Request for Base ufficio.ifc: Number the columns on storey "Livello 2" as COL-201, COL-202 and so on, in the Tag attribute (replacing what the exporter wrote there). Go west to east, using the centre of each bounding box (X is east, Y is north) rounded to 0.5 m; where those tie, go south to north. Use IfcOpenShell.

First a look at what the model holds.

```python
import ifcopenshell
import ifcopenshell.util.element
import ifcopenshell.util.placement

model = ifcopenshell.open("Base ufficio.ifc")
print(model.schema)
storey = next(s for s in model.by_type("IfcBuildingStorey") if s.Name == "Livello 2")
columns = [e for e in ifcopenshell.util.element.get_decomposition(storey) if e.is_a("IfcColumn")]
for e in sorted(columns, key=lambda e: e.id()):
    origin = ifcopenshell.util.placement.get_local_placement(e.ObjectPlacement)[:3, 3]
    print(e.id(), e.Tag, e.Name, origin.round(2) + 0.0, sep=" | ")
```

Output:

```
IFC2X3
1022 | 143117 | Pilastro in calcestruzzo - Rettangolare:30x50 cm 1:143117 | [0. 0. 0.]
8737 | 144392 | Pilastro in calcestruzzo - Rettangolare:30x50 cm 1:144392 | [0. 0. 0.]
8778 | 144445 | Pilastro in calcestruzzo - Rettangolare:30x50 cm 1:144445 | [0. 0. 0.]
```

```python
import ifcopenshell
import ifcopenshell.geom
import ifcopenshell.util.element
import ifcopenshell.util.shape

model = ifcopenshell.open("Base ufficio.ifc")
settings = ifcopenshell.geom.settings()
settings.set("use-world-coords", True)


def centre(element):
    shape = ifcopenshell.geom.create_shape(settings, element)
    return ifcopenshell.util.shape.get_bbox_centroid(shape.geometry)


storey = next(s for s in model.by_type("IfcBuildingStorey") if s.Name == "Livello 2")
columns = [e for e in ifcopenshell.util.element.get_decomposition(storey) if e.is_a("IfcColumn")]

# Insertion points can sit at a corner or the storey origin, so sort by the geometry (in metres).
centres = {e: centre(e) for e in columns}
columns.sort(key=lambda e: (round(centres[e][0] / 0.5), centres[e][1]))

for i, e in enumerate(columns, start=1):
    number = f"COL-2{i:02d}"
    e.Tag = number
    print(e.id(), number)

model.write("Base ufficio_rev.ifc")
```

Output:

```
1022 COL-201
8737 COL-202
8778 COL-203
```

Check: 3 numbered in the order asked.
